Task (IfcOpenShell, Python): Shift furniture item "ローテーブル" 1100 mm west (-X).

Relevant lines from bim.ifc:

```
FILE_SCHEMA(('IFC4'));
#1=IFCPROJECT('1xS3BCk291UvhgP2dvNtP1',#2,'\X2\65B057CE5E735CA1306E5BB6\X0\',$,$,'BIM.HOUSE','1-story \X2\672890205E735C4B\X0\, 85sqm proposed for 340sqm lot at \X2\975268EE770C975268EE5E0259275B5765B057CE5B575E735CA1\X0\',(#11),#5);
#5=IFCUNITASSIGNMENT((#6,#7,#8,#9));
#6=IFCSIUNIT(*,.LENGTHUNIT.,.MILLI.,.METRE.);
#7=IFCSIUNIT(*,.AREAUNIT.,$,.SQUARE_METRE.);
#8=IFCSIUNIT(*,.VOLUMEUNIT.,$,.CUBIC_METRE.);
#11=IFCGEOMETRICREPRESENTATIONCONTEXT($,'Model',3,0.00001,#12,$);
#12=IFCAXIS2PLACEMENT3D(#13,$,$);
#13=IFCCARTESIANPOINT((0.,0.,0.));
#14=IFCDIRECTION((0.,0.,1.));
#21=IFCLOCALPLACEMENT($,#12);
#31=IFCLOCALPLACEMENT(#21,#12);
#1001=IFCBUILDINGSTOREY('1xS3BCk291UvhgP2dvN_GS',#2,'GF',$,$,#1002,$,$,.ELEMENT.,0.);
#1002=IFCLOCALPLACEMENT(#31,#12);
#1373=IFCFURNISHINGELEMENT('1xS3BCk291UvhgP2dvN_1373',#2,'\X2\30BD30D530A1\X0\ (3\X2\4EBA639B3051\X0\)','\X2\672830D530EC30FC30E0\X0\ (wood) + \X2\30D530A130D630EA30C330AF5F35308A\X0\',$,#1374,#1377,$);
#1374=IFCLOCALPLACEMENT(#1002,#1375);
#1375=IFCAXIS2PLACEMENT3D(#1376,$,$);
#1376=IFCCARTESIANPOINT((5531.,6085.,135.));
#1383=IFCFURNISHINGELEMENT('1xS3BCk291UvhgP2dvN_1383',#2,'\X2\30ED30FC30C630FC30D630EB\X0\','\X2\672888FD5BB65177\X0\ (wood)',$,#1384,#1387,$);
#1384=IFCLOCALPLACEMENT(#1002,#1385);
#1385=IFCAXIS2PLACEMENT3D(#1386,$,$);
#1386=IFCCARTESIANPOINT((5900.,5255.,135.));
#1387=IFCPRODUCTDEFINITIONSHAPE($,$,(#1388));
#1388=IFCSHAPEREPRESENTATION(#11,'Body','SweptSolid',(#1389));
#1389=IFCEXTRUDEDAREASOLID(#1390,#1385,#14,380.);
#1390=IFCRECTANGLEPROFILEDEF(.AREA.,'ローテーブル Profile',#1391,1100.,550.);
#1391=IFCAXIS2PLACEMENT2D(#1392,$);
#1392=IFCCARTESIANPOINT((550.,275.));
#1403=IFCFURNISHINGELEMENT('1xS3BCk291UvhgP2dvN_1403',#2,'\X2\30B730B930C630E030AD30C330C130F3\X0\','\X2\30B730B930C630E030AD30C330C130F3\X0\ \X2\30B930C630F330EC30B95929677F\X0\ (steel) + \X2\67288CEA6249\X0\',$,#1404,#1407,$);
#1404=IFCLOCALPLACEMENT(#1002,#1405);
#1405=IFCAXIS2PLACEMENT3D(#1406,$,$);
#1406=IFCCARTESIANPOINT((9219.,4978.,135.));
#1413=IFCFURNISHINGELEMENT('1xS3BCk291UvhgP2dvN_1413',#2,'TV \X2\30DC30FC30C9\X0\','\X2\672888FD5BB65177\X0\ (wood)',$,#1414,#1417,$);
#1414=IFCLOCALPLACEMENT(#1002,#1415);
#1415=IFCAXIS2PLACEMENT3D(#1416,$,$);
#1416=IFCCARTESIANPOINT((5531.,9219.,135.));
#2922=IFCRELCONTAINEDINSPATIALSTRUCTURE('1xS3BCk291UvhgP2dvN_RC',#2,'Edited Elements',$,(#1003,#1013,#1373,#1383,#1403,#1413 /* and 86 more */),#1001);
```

```python
import ifcopenshell
import ifcopenshell.api.geometry
import ifcopenshell.util.placement
import ifcopenshell.util.unit

model = ifcopenshell.open("bim.ifc")
unit_scale = ifcopenshell.util.unit.calculate_unit_scale(model)

item = model.by_guid("1xS3BCk291UvhgP2dvN_1383")
matrix = ifcopenshell.util.placement.get_local_placement(item.ObjectPlacement)
matrix[0, 3] -= 1.1 / unit_scale
ifcopenshell.api.geometry.edit_object_placement(model, product=item, matrix=matrix, is_si=False)

print(ifcopenshell.util.placement.get_local_placement(item.ObjectPlacement).round(3) + 0.0)

model.write("bim_rev.ifc")
```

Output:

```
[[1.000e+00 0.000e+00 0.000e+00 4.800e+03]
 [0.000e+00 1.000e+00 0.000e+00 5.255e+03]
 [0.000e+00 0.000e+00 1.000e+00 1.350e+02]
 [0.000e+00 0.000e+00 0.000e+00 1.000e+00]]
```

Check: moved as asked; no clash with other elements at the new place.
